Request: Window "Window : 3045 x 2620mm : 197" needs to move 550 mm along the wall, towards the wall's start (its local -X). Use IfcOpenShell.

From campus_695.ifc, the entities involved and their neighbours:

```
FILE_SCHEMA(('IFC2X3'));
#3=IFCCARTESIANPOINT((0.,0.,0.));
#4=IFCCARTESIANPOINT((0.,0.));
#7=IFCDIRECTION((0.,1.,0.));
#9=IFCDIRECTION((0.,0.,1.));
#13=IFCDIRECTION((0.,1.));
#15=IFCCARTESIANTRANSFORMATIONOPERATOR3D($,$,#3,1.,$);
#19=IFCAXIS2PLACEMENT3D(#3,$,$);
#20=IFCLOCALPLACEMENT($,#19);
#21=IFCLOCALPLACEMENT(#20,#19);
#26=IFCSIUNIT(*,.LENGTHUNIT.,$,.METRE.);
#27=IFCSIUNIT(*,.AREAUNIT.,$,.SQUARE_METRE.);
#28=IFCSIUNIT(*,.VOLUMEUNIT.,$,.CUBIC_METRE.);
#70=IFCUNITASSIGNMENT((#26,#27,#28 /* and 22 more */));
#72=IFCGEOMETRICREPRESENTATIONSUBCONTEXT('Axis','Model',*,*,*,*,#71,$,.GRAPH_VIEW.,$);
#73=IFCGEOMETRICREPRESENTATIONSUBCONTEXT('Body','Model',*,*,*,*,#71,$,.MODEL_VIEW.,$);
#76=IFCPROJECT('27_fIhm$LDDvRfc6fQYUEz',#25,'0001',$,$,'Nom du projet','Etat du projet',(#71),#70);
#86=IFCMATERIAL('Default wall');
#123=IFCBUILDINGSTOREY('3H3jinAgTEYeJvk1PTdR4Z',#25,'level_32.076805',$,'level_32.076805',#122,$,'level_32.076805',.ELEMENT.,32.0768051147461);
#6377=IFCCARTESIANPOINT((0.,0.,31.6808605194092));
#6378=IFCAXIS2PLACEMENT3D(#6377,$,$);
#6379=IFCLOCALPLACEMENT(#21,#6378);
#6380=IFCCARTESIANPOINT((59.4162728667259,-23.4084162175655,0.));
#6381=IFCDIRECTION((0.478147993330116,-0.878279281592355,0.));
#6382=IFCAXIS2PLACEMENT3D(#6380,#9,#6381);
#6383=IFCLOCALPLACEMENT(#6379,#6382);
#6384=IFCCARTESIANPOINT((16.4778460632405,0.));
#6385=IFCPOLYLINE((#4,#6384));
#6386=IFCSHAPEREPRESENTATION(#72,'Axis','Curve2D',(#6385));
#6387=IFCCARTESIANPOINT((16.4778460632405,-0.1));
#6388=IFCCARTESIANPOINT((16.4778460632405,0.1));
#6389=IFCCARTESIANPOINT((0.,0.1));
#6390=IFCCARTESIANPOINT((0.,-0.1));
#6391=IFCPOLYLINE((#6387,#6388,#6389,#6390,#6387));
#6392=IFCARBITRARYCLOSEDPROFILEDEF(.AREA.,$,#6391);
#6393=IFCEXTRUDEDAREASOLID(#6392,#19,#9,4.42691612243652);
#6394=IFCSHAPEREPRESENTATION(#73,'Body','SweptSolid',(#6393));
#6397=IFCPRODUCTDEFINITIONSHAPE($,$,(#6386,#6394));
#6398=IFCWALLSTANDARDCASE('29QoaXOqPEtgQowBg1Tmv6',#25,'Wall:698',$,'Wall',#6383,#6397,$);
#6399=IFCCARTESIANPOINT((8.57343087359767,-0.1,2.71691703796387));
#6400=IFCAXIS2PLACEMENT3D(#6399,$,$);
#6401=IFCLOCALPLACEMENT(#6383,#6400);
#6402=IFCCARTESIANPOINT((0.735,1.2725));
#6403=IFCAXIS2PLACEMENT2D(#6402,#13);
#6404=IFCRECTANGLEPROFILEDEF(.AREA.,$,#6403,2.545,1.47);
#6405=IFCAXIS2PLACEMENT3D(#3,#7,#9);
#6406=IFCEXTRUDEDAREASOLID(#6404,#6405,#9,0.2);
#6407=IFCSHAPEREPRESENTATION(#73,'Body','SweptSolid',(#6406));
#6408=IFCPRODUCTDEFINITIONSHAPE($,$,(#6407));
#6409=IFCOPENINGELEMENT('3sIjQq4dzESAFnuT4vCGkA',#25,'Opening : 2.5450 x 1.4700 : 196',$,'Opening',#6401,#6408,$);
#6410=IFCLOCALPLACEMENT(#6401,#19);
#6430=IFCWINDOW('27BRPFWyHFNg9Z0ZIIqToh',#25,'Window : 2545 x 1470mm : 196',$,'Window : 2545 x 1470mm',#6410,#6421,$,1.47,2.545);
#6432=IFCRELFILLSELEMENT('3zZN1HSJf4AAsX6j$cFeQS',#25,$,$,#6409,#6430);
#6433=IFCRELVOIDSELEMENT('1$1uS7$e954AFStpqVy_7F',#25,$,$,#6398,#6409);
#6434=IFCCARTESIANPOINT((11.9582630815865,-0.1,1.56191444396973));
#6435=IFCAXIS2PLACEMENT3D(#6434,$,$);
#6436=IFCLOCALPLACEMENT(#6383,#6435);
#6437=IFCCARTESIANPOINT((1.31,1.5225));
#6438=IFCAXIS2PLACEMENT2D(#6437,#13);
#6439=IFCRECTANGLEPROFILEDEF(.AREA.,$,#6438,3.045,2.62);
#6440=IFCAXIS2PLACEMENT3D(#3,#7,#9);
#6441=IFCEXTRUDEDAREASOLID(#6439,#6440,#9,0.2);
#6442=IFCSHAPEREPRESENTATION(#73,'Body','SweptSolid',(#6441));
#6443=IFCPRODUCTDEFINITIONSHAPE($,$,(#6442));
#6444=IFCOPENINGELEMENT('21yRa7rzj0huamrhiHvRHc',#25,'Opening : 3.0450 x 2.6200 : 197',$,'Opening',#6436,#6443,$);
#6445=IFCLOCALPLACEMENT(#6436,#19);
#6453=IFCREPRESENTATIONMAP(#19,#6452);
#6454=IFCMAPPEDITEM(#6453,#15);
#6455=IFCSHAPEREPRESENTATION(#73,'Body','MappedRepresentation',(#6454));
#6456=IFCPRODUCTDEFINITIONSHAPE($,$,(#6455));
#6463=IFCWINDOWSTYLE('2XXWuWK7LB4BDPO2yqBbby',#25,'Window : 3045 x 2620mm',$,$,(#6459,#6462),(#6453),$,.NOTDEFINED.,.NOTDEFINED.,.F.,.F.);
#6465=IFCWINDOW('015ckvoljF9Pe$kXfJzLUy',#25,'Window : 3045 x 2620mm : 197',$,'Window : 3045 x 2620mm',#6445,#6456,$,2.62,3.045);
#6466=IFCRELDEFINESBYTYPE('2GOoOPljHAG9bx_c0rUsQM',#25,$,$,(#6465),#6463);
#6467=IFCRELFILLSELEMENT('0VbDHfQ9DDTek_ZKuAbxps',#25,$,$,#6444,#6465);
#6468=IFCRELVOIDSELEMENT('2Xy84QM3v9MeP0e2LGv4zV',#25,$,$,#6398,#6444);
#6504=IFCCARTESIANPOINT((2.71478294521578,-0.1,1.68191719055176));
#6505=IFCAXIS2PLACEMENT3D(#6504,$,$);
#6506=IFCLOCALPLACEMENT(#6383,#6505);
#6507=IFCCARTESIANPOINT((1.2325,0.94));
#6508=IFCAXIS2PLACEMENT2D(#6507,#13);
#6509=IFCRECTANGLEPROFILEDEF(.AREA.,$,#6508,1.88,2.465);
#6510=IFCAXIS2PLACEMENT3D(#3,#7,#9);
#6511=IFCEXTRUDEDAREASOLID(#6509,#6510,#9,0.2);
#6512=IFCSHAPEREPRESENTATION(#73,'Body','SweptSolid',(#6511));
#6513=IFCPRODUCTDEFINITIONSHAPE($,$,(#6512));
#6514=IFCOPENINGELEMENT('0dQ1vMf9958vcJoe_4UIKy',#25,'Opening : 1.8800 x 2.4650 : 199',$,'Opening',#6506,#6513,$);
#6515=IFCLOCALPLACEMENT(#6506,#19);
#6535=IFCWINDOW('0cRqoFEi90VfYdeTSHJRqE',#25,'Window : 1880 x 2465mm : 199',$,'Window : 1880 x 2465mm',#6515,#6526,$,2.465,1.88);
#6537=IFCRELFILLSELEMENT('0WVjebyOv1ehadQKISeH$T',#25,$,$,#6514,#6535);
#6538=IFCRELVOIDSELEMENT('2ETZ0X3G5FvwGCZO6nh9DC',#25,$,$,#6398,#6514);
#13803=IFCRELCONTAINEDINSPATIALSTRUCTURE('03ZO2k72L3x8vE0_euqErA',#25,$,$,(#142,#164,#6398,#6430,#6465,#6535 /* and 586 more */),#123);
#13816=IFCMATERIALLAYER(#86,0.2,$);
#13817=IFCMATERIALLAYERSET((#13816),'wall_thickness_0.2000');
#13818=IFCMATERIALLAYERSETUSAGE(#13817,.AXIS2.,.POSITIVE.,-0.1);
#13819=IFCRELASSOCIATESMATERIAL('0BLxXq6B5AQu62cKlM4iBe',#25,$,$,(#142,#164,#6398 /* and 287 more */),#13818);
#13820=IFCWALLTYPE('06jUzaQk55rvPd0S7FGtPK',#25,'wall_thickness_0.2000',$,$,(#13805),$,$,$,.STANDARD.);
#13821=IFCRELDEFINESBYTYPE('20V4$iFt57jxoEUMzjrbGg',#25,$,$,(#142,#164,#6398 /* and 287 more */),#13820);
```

```python
import ifcopenshell
import ifcopenshell.api.geometry
import ifcopenshell.util.placement
import ifcopenshell.util.unit

model = ifcopenshell.open("campus_695.ifc")
unit_scale = ifcopenshell.util.unit.calculate_unit_scale(model)

window = model.by_guid("015ckvoljF9Pe$kXfJzLUy")
opening = window.FillsVoids[0].RelatingOpeningElement
wall = opening.VoidsElements[0].RelatingBuildingElement

wall_matrix = ifcopenshell.util.placement.get_local_placement(wall.ObjectPlacement)
shift = wall_matrix[:3, 0] * -0.55 / unit_scale
before = ifcopenshell.util.placement.get_local_placement(window.ObjectPlacement)[:3, 3].copy()

# The window is placed relative to its opening, so it follows when the opening moves.
matrix = ifcopenshell.util.placement.get_local_placement(opening.ObjectPlacement)
matrix[:3, 3] += shift
ifcopenshell.api.geometry.edit_object_placement(
    model, product=opening, matrix=matrix, is_si=False, should_transform_children=True
)

after = ifcopenshell.util.placement.get_local_placement(window.ObjectPlacement)[:3, 3]
print("window moved by", (after - before).round(3) + 0.0)

model.write("campus_695_rev.ifc")
```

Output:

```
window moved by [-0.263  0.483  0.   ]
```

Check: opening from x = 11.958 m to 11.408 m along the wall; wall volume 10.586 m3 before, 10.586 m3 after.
